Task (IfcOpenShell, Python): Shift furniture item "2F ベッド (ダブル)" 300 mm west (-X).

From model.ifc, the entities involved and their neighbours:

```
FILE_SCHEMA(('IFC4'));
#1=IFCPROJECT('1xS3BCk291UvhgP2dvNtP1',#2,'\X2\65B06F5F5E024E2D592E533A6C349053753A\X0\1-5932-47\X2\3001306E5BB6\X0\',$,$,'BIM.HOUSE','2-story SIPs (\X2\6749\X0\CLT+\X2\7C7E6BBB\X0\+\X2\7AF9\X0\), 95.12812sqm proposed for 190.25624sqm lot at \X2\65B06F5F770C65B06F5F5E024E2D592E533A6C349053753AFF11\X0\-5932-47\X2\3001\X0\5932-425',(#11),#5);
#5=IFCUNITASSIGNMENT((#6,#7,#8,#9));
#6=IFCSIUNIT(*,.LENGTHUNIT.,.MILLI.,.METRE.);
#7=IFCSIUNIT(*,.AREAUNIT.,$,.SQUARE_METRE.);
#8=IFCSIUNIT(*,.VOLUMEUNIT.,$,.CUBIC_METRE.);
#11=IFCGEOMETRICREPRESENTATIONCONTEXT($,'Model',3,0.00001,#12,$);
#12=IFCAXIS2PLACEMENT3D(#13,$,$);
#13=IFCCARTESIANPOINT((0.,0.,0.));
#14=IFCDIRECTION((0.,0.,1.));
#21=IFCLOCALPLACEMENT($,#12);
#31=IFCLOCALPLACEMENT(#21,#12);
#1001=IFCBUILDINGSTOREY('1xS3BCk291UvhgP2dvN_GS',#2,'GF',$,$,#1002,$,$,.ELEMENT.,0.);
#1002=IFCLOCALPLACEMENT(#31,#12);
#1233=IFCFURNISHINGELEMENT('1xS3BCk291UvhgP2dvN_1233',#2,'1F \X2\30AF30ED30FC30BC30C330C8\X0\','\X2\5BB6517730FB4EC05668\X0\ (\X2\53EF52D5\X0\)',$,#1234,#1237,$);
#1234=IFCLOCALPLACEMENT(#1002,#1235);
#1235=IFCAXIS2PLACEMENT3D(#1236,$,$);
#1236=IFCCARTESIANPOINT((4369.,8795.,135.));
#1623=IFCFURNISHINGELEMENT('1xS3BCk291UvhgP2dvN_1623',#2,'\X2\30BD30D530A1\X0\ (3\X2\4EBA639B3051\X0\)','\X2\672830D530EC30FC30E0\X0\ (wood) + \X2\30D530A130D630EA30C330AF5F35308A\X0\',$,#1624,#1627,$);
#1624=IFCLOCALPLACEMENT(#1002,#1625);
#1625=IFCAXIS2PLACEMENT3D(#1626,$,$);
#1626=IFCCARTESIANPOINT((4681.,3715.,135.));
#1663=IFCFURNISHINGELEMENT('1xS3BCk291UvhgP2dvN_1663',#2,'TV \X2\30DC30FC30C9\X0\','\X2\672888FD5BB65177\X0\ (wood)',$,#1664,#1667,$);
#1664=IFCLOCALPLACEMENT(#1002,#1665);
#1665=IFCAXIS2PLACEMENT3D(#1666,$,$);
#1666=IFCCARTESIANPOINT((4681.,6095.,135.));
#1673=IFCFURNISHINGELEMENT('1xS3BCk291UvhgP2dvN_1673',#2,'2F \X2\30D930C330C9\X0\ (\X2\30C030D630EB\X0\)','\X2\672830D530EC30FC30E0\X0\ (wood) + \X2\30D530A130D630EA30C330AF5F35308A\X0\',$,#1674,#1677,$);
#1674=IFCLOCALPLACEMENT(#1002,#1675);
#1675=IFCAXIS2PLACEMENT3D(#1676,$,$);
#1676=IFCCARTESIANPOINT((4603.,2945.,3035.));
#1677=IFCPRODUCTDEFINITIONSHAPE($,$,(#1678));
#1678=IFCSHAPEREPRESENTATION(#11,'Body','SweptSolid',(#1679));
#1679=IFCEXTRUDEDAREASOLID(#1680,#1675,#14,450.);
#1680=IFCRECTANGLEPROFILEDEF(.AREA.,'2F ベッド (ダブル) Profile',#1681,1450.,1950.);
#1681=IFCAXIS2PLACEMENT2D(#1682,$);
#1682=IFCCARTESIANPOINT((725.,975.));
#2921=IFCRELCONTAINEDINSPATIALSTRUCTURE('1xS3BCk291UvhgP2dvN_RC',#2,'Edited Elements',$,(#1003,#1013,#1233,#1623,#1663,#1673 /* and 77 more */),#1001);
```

```python
import ifcopenshell
import ifcopenshell.api.geometry
import ifcopenshell.util.placement

model = ifcopenshell.open("model.ifc")

item = model.by_guid("1xS3BCk291UvhgP2dvN_1673")
matrix = ifcopenshell.util.placement.get_local_placement(item.ObjectPlacement)
matrix[0, 3] -= 300.0
ifcopenshell.api.geometry.edit_object_placement(model, product=item, matrix=matrix, is_si=False)

print(ifcopenshell.util.placement.get_local_placement(item.ObjectPlacement).round(3) + 0.0)

model.write("model_v2.ifc")
```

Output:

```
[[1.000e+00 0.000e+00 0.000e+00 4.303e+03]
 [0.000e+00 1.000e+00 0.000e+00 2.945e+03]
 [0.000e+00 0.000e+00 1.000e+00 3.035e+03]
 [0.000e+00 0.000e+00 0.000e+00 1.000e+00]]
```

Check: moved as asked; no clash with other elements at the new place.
